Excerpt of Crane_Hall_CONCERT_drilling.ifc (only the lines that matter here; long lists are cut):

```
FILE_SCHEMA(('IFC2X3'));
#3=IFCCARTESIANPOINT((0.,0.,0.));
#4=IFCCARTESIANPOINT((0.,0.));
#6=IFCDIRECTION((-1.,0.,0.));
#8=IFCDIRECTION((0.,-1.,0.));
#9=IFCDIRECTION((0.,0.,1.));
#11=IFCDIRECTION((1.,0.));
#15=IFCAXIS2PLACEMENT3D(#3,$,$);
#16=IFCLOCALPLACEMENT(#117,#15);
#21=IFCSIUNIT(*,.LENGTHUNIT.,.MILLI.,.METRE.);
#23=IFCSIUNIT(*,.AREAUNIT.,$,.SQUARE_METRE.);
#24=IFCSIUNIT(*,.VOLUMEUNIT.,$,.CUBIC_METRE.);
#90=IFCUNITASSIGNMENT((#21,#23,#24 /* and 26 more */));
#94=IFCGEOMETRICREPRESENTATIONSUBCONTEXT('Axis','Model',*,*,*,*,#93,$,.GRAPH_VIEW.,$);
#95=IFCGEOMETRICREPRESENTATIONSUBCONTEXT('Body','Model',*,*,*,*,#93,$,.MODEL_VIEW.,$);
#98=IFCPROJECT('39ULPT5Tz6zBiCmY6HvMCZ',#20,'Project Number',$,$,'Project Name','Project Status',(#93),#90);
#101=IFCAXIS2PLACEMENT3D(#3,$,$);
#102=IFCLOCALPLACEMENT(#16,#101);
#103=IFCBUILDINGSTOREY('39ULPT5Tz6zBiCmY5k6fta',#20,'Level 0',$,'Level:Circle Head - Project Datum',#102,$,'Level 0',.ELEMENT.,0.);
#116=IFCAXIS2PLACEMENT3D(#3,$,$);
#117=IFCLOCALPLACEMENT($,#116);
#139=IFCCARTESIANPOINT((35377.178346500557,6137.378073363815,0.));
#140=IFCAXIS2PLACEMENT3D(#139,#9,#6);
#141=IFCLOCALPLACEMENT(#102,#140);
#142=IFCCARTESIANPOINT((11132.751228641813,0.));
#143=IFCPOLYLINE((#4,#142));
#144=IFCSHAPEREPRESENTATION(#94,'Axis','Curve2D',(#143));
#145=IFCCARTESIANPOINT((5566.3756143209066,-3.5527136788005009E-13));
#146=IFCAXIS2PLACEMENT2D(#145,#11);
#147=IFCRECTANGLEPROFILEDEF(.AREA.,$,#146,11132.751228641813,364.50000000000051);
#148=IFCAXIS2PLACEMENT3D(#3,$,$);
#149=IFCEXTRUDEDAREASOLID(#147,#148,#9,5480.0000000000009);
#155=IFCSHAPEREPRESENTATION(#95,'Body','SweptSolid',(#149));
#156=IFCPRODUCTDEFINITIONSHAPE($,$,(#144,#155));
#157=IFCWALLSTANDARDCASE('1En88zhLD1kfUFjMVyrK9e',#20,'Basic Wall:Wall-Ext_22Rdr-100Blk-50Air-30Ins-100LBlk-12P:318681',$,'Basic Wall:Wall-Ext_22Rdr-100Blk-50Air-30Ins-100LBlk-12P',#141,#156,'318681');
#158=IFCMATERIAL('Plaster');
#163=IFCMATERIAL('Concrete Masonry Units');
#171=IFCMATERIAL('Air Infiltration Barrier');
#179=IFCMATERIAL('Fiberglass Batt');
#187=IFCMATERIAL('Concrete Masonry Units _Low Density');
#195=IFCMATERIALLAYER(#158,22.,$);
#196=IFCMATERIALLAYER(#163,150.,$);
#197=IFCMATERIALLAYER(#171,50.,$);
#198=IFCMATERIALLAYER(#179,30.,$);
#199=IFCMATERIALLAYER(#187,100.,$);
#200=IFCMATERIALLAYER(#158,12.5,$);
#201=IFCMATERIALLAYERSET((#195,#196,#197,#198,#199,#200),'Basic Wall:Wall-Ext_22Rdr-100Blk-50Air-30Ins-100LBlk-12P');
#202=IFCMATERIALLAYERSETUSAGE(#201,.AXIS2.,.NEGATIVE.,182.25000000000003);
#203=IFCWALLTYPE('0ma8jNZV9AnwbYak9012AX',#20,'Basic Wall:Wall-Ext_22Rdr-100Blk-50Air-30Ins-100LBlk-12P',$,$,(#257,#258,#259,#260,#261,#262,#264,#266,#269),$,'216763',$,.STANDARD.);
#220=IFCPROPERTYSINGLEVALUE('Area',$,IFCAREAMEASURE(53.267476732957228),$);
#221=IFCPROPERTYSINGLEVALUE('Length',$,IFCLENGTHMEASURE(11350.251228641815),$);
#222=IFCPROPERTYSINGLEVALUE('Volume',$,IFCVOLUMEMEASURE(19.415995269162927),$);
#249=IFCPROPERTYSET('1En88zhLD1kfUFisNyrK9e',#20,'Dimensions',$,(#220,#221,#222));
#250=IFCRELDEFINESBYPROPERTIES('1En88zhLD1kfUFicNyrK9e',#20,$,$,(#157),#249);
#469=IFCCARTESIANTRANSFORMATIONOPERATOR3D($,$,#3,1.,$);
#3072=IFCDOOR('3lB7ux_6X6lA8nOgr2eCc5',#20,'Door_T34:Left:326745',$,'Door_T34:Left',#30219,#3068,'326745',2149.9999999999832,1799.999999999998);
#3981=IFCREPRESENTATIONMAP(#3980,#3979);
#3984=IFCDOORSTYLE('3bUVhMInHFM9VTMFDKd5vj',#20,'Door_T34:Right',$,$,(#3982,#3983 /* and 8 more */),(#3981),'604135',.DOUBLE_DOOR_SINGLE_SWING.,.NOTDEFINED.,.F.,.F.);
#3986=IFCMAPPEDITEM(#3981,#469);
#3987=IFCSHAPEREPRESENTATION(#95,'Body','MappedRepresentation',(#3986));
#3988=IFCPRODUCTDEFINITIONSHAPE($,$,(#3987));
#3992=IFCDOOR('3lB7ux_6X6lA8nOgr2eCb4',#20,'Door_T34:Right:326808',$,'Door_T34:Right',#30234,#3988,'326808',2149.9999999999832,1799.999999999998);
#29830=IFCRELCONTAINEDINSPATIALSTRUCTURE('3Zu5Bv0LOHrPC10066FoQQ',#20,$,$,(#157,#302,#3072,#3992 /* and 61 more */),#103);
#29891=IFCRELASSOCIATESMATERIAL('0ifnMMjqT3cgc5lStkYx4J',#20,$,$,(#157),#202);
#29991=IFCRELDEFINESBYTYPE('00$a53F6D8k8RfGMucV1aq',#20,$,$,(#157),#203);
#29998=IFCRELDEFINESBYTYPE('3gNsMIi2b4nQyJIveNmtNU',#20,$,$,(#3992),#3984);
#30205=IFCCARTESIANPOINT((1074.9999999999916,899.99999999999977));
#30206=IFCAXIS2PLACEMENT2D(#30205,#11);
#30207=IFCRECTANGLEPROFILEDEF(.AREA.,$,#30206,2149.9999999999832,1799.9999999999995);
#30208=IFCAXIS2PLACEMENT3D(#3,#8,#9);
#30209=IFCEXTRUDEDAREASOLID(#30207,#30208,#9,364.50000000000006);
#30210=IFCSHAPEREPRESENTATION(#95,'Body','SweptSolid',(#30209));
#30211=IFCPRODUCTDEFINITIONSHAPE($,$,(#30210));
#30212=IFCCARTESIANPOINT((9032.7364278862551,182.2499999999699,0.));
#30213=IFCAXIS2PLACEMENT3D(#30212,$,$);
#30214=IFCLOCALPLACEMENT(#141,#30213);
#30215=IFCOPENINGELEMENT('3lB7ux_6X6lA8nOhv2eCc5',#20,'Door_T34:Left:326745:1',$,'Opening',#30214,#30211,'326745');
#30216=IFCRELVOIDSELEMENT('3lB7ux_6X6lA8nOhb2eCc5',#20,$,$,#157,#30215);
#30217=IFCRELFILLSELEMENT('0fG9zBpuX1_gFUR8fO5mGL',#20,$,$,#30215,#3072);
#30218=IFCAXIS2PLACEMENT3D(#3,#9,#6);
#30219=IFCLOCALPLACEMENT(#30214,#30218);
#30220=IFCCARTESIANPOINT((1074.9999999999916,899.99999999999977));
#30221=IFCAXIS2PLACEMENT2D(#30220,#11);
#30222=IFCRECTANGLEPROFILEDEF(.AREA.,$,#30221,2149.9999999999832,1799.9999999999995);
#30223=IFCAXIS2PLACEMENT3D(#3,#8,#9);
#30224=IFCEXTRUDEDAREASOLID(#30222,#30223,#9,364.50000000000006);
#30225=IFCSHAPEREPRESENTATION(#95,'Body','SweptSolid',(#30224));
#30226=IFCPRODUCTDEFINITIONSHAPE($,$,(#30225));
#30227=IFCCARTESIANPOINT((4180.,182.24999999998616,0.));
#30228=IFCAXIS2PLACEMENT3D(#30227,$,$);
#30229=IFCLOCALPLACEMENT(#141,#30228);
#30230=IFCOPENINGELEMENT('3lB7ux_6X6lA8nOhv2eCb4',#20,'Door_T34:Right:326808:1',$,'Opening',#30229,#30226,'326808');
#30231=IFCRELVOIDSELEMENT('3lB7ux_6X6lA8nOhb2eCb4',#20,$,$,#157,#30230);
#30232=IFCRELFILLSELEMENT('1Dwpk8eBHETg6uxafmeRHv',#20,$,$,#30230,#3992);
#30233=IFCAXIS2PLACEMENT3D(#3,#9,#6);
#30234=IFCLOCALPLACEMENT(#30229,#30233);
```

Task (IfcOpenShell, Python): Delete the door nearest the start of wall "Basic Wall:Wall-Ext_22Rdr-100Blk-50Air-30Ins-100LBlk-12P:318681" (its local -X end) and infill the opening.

```python
import ifcopenshell
import ifcopenshell.api.feature
import ifcopenshell.api.pset
import ifcopenshell.api.root
import ifcopenshell.geom
import ifcopenshell.util.element
import ifcopenshell.util.shape
import ifcopenshell.util.unit

model = ifcopenshell.open("Crane_Hall_CONCERT_drilling.ifc")
area_scale = ifcopenshell.util.unit.calculate_unit_scale(model, "AREAUNIT")
volume_scale = ifcopenshell.util.unit.calculate_unit_scale(model, "VOLUMEUNIT")
settings = ifcopenshell.geom.settings()


def volume(element):
    """Net volume in cubic metres, openings subtracted."""
    shape = ifcopenshell.geom.create_shape(settings, element)
    return ifcopenshell.util.shape.get_volume(shape.geometry)


door = model.by_guid("3lB7ux_6X6lA8nOgr2eCb4")
opening = door.FillsVoids[0].RelatingOpeningElement
wall = opening.VoidsElements[0].RelatingBuildingElement
before = volume(wall)

ifcopenshell.api.root.remove_product(model, product=door)
ifcopenshell.api.feature.remove_feature(model, feature=opening)

after = volume(wall)
thickness = 0.3645  # wall thickness in metres

# Update the wall's stored quantities.
pset = model.by_id(ifcopenshell.util.element.get_pset(wall, "Dimensions", should_inherit=False)["id"])
ifcopenshell.api.pset.edit_pset(model, pset=pset, properties={
    "Area": model.create_entity("IfcAreaMeasure", after / thickness / area_scale),
    "Volume": model.create_entity("IfcVolumeMeasure", after / volume_scale),
})

print(f"wall volume {before:.3f} -> {after:.3f} m3")

model.write("Crane_Hall_CONCERT_drilling-out.ifc")
```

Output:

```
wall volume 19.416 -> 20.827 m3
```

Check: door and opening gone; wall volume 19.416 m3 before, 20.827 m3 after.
